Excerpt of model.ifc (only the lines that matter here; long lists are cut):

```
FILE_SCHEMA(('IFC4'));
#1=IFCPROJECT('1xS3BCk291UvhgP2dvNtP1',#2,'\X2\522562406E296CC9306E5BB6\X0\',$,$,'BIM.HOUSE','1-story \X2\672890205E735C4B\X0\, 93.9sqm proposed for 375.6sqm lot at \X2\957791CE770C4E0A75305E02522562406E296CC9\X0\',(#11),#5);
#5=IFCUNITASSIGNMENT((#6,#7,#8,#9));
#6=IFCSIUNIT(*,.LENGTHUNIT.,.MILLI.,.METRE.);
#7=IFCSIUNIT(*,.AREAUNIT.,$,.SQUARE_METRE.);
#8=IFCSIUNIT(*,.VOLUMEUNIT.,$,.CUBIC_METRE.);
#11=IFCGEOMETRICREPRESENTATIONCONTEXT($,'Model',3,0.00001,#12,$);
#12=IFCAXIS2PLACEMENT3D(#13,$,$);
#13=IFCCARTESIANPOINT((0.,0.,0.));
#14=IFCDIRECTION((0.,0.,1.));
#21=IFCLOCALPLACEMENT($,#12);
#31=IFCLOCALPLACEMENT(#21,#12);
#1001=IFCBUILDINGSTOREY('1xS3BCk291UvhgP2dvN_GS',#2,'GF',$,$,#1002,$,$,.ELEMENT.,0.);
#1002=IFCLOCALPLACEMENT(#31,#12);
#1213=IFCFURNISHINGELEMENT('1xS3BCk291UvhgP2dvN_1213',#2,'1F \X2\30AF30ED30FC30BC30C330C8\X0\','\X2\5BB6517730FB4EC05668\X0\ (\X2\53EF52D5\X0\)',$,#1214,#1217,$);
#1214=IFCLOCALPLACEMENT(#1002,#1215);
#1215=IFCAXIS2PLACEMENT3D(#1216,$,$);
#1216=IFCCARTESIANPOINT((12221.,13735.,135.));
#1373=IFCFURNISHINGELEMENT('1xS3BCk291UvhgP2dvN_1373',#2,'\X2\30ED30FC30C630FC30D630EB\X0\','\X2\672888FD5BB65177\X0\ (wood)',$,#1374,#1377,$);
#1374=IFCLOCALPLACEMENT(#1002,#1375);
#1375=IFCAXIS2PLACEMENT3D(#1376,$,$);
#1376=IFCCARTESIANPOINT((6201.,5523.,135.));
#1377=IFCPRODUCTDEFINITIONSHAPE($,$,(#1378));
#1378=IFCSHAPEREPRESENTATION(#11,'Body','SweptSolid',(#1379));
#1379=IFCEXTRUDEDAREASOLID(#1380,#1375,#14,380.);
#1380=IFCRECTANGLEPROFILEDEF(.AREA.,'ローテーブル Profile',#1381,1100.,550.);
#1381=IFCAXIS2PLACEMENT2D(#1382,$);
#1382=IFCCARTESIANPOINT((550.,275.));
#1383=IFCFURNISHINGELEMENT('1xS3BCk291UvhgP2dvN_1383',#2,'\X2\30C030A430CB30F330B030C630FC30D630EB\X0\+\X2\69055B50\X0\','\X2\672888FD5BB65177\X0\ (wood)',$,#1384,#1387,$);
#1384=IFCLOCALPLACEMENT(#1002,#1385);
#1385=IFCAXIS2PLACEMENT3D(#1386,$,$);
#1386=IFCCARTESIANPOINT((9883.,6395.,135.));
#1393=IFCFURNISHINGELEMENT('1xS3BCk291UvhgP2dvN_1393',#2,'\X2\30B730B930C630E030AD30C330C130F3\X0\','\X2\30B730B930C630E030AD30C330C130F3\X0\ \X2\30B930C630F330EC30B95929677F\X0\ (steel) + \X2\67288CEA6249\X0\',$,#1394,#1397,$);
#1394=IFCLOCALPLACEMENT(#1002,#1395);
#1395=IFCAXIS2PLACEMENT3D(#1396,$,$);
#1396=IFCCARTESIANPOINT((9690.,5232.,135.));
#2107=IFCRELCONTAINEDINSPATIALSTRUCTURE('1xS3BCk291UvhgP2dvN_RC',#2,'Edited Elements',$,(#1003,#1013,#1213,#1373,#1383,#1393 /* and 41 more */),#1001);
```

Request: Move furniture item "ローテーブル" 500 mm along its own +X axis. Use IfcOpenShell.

```python
import ifcopenshell
import ifcopenshell.api.geometry
import ifcopenshell.util.placement
import ifcopenshell.util.unit

model = ifcopenshell.open("model.ifc")
unit_scale = ifcopenshell.util.unit.calculate_unit_scale(model)

item = model.by_guid("1xS3BCk291UvhgP2dvN_1373")
matrix = ifcopenshell.util.placement.get_local_placement(item.ObjectPlacement)
matrix[:3, 3] += matrix[:3, 0] * 0.5 / unit_scale
ifcopenshell.api.geometry.edit_object_placement(model, product=item, matrix=matrix, is_si=False)

print(ifcopenshell.util.placement.get_local_placement(item.ObjectPlacement).round(3) + 0.0)

model.write("model_rev.ifc")
```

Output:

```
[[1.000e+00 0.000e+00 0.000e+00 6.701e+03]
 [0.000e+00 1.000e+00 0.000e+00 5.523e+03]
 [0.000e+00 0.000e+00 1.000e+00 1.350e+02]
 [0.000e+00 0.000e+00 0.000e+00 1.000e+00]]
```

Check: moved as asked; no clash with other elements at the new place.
